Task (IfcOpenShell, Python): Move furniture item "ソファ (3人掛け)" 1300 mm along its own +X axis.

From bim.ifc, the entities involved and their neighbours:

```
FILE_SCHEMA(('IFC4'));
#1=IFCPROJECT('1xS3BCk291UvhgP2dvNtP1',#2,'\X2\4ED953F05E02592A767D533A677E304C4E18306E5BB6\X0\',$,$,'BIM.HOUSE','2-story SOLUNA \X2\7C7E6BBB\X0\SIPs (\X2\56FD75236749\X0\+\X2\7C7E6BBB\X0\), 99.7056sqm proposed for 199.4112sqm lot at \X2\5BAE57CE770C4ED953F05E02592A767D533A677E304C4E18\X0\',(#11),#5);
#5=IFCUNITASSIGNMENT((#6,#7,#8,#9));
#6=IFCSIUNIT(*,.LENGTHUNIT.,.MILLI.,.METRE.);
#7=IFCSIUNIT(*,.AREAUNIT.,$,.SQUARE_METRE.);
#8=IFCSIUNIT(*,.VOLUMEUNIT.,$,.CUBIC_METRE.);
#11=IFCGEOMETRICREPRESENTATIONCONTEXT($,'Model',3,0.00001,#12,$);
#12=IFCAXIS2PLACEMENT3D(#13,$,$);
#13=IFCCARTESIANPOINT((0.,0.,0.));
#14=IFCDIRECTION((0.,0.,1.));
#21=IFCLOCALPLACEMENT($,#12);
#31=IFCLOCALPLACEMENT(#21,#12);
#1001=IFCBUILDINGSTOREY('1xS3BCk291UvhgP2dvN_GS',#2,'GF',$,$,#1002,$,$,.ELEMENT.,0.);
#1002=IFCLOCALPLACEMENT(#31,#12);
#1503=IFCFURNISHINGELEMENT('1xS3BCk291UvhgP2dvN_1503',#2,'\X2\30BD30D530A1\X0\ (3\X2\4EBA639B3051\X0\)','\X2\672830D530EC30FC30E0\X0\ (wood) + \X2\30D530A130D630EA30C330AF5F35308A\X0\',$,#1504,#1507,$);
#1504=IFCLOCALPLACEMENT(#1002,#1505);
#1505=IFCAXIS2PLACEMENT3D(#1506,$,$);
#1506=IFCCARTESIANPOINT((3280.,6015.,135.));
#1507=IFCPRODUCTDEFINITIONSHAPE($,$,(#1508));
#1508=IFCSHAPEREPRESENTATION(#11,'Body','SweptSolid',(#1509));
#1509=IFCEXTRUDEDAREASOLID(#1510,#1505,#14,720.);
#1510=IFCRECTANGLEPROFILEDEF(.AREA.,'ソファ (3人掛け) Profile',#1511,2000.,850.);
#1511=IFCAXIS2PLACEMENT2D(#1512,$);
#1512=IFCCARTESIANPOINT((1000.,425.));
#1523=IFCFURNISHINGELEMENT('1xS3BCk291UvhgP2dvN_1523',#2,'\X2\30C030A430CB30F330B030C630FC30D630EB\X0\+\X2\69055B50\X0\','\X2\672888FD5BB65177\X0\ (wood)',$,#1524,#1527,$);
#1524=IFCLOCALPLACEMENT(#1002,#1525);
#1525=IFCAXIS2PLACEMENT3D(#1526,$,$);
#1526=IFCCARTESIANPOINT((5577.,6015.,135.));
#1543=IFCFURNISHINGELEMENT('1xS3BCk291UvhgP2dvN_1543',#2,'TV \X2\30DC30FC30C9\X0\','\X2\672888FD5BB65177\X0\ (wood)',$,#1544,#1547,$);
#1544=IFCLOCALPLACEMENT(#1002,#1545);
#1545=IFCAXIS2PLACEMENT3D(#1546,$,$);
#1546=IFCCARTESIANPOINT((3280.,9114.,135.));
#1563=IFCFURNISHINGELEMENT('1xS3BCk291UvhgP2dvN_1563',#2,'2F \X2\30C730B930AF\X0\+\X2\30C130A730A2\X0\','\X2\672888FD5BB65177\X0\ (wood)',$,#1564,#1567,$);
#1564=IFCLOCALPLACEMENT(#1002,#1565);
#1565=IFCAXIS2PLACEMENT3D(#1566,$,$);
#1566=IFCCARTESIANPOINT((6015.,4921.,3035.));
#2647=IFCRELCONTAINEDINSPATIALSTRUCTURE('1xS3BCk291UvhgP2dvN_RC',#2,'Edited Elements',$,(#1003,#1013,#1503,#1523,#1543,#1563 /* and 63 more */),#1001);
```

```python
import ifcopenshell
import ifcopenshell.api.geometry
import ifcopenshell.util.placement
import ifcopenshell.util.unit

model = ifcopenshell.open("bim.ifc")
unit_scale = ifcopenshell.util.unit.calculate_unit_scale(model)

item = model.by_guid("1xS3BCk291UvhgP2dvN_1503")
matrix = ifcopenshell.util.placement.get_local_placement(item.ObjectPlacement)
matrix[:3, 3] += matrix[:3, 0] * 1.3 / unit_scale
ifcopenshell.api.geometry.edit_object_placement(model, product=item, matrix=matrix, is_si=False)

print(ifcopenshell.util.placement.get_local_placement(item.ObjectPlacement).round(3) + 0.0)

model.write("bim_v2.ifc")
```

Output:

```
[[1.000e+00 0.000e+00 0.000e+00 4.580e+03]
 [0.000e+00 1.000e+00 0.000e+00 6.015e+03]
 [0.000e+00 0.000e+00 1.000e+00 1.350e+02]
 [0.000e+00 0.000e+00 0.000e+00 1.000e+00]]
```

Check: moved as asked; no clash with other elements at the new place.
